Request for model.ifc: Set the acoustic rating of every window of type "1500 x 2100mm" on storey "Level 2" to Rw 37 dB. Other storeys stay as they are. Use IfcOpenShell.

First a look at what the model holds.

```python
import ifcopenshell
import ifcopenshell.util.element

model = ifcopenshell.open("model.ifc")
print(model.schema)
storey = next(s for s in model.by_type("IfcBuildingStorey") if s.Name == "Level 2")
windows = [e for e in ifcopenshell.util.element.get_decomposition(storey) if e.is_a("IfcWindow")]
seen = {}
for e in windows:
    element_type = ifcopenshell.util.element.get_type(e)
    key = (element_type.Name if element_type != e and element_type else None, ifcopenshell.util.element.get_pset(e, "Pset_WindowCommon", "AcousticRating"))
    seen[key] = seen.get(key, 0) + 1
for (name, value), count in sorted(seen.items(), key=str):
    print(count, "x", name, "|", value)
```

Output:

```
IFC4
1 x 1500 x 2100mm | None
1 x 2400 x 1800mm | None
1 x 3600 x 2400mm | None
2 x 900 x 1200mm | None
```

```python
import ifcopenshell
import ifcopenshell.api.pset
import ifcopenshell.util.element

model = ifcopenshell.open("model.ifc")

storey = next(s for s in model.by_type("IfcBuildingStorey") if s.Name == "Level 2")
windows = [e for e in ifcopenshell.util.element.get_decomposition(storey) if e.is_a("IfcWindow")]

count = 0
for e in windows:
    element_type = ifcopenshell.util.element.get_type(e)
    if element_type in (None, e) or element_type.Name != "1500 x 2100mm":
        continue
    # add_pset returns the element's existing set when there is one.
    pset = ifcopenshell.api.pset.add_pset(model, product=e, name="Pset_WindowCommon")
    ifcopenshell.api.pset.edit_pset(model, pset=pset, properties={"AcousticRating": "Rw 37 dB"})
    count += 1

print(count, "windows updated")

model.write("model_v2.ifc")
```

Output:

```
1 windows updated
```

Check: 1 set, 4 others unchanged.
